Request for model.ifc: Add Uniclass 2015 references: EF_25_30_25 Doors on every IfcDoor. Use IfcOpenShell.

First a look at what the model holds.

```python
import ifcopenshell

model = ifcopenshell.open("model.ifc")
print(model.schema)
print("classifications:", [c.Name for c in model.by_type("IfcClassification")])
for ifc_class in ("IfcDoor", "IfcRoof", "IfcStair", "IfcWall", "IfcWindow"):
    print(ifc_class, len(model.by_type(ifc_class)))
```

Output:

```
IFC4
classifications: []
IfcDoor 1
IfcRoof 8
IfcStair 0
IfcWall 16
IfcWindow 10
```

```python
import ifcopenshell
import ifcopenshell.api.classification

model = ifcopenshell.open("model.ifc")

system = ifcopenshell.api.classification.add_classification(model, classification="Uniclass 2015")

codes = {
    "IfcDoor": ("EF_25_30_25", "Doors"),
}
for ifc_class, (code, name) in codes.items():
    products = model.by_type(ifc_class)
    ifcopenshell.api.classification.add_reference(
        model, products=products, classification=system, identification=code, name=name
    )
    print(code, len(products))

model.write("model_updated.ifc")
```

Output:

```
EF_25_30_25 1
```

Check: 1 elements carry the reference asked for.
